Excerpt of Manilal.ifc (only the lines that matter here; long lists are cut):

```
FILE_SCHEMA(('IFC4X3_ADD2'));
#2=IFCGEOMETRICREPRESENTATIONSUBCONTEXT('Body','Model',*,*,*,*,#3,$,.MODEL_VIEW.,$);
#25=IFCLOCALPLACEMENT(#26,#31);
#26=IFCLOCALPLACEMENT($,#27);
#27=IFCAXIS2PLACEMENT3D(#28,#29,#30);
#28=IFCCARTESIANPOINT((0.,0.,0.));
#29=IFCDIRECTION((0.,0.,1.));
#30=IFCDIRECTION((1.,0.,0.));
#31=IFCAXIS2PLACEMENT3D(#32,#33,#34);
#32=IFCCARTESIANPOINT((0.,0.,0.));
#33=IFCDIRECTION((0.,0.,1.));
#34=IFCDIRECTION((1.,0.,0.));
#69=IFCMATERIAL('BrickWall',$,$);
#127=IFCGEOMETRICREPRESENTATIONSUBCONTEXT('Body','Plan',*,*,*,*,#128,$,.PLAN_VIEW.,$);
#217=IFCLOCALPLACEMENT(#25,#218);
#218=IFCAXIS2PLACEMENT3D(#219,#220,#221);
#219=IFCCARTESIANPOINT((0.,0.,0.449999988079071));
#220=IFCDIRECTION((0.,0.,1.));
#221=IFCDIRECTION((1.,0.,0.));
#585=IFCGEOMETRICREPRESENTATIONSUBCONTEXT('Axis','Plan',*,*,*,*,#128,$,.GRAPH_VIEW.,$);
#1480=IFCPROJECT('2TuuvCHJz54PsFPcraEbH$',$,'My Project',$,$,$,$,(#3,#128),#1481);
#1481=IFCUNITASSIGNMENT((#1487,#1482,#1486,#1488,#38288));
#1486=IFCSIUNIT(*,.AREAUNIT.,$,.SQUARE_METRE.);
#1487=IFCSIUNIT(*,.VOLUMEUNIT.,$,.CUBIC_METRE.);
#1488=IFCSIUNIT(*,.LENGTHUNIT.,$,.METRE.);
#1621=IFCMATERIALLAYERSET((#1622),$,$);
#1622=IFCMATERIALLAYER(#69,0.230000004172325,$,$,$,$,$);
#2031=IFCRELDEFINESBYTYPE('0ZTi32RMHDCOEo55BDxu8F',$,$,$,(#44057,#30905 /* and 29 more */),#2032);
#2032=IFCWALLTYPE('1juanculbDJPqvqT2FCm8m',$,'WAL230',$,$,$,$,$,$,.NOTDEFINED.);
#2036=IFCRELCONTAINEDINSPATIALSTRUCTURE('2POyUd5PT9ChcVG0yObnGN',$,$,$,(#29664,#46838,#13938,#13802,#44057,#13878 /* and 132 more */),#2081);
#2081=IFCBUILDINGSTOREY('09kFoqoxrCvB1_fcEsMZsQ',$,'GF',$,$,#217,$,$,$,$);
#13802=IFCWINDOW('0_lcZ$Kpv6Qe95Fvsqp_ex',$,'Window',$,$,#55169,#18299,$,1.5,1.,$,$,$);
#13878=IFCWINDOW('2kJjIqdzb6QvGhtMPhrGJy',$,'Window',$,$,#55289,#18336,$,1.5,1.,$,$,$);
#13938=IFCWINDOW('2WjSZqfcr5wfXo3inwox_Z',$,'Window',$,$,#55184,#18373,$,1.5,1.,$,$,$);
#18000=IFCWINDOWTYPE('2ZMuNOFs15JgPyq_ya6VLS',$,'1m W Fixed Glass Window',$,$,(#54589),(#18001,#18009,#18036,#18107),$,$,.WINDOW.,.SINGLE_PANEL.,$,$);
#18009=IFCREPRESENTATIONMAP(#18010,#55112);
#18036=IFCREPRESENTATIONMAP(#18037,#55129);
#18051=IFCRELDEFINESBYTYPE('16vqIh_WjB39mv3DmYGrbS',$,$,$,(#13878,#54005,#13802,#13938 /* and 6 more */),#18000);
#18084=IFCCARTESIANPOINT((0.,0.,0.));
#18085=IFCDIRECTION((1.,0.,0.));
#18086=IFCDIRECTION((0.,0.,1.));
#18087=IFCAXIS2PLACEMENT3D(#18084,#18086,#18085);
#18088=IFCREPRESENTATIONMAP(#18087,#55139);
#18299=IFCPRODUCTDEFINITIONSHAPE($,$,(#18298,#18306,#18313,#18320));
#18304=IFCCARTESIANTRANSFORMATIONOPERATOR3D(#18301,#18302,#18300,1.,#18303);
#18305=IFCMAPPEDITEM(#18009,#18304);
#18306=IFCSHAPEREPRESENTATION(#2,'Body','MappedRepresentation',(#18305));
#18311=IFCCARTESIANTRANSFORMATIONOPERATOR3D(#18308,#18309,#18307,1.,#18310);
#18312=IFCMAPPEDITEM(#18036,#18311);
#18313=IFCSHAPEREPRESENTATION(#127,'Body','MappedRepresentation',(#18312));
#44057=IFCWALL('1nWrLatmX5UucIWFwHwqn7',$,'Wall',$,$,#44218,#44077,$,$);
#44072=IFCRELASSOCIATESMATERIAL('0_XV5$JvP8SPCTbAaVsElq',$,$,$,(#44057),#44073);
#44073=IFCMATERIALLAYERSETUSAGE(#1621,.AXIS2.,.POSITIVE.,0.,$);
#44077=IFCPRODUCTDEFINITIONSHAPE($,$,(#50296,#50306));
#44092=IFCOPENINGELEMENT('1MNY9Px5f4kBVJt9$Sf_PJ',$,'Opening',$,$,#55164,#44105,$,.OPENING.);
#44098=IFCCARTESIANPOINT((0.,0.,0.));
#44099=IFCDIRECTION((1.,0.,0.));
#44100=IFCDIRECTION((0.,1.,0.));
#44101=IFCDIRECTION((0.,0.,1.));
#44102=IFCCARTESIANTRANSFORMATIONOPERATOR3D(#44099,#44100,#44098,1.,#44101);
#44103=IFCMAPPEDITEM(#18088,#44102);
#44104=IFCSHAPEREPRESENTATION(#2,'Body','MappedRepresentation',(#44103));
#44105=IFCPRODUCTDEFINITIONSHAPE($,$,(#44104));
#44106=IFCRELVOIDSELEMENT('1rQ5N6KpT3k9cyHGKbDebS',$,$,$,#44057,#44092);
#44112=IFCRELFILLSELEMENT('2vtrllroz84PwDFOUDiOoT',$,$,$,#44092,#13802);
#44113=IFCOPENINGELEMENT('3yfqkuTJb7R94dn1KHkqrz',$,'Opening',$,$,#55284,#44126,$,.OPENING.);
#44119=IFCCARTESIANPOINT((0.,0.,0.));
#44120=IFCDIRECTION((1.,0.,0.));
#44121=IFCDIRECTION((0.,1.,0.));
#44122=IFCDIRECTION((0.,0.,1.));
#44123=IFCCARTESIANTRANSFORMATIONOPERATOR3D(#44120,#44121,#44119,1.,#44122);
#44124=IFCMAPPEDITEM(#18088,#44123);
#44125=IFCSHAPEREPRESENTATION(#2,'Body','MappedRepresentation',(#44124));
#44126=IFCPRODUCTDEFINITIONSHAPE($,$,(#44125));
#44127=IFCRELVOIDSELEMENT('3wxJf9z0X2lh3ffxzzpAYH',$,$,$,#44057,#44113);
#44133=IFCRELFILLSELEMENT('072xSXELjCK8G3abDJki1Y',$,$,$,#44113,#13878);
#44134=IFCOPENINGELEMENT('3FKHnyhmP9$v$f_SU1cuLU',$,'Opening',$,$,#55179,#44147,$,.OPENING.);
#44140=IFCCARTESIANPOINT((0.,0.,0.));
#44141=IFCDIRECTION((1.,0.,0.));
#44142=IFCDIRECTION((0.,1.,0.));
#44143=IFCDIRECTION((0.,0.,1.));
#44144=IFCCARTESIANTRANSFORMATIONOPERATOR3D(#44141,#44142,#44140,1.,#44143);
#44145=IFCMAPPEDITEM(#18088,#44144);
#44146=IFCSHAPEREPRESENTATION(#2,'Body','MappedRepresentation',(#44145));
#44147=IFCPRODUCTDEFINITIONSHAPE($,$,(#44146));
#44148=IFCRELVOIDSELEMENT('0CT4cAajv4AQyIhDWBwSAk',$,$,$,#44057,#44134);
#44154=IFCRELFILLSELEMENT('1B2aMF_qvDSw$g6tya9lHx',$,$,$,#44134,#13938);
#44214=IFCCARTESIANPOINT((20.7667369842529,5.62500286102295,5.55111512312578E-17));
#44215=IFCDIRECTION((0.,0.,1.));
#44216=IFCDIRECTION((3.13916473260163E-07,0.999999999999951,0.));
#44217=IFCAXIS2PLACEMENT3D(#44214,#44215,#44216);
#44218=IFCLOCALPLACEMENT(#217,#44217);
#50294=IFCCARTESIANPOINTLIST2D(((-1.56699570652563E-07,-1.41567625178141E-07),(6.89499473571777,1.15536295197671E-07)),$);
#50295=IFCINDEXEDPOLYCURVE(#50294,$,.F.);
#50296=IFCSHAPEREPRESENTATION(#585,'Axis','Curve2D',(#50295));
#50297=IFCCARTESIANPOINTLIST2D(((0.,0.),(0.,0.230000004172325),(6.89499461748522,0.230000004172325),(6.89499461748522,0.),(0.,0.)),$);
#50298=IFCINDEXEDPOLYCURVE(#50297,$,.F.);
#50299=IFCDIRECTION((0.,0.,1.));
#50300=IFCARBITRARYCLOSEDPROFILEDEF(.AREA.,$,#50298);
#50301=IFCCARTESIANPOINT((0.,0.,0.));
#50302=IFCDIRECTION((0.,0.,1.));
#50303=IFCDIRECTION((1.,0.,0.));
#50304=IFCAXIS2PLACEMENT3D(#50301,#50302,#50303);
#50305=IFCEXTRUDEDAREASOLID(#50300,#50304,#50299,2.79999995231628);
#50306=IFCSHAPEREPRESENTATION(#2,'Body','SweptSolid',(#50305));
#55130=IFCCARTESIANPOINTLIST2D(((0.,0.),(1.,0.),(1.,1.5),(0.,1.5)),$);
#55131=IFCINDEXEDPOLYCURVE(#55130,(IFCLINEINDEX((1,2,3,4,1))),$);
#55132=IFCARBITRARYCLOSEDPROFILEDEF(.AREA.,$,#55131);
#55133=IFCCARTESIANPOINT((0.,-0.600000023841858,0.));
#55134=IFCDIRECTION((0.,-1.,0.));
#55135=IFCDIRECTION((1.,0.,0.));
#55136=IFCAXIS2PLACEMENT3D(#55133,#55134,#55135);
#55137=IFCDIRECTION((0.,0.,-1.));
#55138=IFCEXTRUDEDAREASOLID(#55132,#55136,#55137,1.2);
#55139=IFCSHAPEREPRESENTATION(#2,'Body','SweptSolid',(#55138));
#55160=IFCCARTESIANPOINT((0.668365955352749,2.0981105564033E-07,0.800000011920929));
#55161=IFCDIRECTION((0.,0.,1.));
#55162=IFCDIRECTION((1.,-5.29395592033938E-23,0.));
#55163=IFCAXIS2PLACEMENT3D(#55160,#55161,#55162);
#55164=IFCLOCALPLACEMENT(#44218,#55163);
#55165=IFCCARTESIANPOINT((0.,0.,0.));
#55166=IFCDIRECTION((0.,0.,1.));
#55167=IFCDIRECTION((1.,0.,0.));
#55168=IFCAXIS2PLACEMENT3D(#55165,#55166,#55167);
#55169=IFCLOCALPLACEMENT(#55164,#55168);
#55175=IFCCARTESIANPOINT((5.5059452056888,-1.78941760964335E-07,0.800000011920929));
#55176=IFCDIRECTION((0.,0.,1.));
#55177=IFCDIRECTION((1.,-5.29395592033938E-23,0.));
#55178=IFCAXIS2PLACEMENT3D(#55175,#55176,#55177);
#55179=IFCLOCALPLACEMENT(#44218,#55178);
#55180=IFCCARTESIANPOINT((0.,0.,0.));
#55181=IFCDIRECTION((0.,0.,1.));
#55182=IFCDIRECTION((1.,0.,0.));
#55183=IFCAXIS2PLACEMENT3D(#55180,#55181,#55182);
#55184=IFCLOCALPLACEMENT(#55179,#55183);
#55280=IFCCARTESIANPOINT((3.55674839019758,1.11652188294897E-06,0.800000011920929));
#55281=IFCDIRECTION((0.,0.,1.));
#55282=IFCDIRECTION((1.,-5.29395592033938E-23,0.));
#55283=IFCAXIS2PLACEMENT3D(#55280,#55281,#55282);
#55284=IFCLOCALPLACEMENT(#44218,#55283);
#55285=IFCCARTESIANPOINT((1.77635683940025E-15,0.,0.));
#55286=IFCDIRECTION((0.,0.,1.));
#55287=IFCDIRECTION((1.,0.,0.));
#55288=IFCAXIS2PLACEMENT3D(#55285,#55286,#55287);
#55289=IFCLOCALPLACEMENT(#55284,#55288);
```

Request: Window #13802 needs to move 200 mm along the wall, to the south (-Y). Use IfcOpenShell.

```python
import ifcopenshell
import ifcopenshell.api.geometry
import ifcopenshell.util.placement
import ifcopenshell.util.unit

model = ifcopenshell.open("Manilal.ifc")
unit_scale = ifcopenshell.util.unit.calculate_unit_scale(model)

window = model.by_id(13802)
opening = window.FillsVoids[0].RelatingOpeningElement
wall = opening.VoidsElements[0].RelatingBuildingElement

wall_matrix = ifcopenshell.util.placement.get_local_placement(wall.ObjectPlacement)
shift = wall_matrix[:3, 0] * -0.2 / unit_scale
before = ifcopenshell.util.placement.get_local_placement(window.ObjectPlacement)[:3, 3].copy()

# The window is placed relative to its opening, so it follows when the opening moves.
matrix = ifcopenshell.util.placement.get_local_placement(opening.ObjectPlacement)
matrix[:3, 3] += shift
ifcopenshell.api.geometry.edit_object_placement(
    model, product=opening, matrix=matrix, is_si=False, should_transform_children=True
)

after = ifcopenshell.util.placement.get_local_placement(window.ObjectPlacement)[:3, 3]
print("window moved by", (after - before).round(3) + 0.0)

model.write("Manilal_updated.ifc")
```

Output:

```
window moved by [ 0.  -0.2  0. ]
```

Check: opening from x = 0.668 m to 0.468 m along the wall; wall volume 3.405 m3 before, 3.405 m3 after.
